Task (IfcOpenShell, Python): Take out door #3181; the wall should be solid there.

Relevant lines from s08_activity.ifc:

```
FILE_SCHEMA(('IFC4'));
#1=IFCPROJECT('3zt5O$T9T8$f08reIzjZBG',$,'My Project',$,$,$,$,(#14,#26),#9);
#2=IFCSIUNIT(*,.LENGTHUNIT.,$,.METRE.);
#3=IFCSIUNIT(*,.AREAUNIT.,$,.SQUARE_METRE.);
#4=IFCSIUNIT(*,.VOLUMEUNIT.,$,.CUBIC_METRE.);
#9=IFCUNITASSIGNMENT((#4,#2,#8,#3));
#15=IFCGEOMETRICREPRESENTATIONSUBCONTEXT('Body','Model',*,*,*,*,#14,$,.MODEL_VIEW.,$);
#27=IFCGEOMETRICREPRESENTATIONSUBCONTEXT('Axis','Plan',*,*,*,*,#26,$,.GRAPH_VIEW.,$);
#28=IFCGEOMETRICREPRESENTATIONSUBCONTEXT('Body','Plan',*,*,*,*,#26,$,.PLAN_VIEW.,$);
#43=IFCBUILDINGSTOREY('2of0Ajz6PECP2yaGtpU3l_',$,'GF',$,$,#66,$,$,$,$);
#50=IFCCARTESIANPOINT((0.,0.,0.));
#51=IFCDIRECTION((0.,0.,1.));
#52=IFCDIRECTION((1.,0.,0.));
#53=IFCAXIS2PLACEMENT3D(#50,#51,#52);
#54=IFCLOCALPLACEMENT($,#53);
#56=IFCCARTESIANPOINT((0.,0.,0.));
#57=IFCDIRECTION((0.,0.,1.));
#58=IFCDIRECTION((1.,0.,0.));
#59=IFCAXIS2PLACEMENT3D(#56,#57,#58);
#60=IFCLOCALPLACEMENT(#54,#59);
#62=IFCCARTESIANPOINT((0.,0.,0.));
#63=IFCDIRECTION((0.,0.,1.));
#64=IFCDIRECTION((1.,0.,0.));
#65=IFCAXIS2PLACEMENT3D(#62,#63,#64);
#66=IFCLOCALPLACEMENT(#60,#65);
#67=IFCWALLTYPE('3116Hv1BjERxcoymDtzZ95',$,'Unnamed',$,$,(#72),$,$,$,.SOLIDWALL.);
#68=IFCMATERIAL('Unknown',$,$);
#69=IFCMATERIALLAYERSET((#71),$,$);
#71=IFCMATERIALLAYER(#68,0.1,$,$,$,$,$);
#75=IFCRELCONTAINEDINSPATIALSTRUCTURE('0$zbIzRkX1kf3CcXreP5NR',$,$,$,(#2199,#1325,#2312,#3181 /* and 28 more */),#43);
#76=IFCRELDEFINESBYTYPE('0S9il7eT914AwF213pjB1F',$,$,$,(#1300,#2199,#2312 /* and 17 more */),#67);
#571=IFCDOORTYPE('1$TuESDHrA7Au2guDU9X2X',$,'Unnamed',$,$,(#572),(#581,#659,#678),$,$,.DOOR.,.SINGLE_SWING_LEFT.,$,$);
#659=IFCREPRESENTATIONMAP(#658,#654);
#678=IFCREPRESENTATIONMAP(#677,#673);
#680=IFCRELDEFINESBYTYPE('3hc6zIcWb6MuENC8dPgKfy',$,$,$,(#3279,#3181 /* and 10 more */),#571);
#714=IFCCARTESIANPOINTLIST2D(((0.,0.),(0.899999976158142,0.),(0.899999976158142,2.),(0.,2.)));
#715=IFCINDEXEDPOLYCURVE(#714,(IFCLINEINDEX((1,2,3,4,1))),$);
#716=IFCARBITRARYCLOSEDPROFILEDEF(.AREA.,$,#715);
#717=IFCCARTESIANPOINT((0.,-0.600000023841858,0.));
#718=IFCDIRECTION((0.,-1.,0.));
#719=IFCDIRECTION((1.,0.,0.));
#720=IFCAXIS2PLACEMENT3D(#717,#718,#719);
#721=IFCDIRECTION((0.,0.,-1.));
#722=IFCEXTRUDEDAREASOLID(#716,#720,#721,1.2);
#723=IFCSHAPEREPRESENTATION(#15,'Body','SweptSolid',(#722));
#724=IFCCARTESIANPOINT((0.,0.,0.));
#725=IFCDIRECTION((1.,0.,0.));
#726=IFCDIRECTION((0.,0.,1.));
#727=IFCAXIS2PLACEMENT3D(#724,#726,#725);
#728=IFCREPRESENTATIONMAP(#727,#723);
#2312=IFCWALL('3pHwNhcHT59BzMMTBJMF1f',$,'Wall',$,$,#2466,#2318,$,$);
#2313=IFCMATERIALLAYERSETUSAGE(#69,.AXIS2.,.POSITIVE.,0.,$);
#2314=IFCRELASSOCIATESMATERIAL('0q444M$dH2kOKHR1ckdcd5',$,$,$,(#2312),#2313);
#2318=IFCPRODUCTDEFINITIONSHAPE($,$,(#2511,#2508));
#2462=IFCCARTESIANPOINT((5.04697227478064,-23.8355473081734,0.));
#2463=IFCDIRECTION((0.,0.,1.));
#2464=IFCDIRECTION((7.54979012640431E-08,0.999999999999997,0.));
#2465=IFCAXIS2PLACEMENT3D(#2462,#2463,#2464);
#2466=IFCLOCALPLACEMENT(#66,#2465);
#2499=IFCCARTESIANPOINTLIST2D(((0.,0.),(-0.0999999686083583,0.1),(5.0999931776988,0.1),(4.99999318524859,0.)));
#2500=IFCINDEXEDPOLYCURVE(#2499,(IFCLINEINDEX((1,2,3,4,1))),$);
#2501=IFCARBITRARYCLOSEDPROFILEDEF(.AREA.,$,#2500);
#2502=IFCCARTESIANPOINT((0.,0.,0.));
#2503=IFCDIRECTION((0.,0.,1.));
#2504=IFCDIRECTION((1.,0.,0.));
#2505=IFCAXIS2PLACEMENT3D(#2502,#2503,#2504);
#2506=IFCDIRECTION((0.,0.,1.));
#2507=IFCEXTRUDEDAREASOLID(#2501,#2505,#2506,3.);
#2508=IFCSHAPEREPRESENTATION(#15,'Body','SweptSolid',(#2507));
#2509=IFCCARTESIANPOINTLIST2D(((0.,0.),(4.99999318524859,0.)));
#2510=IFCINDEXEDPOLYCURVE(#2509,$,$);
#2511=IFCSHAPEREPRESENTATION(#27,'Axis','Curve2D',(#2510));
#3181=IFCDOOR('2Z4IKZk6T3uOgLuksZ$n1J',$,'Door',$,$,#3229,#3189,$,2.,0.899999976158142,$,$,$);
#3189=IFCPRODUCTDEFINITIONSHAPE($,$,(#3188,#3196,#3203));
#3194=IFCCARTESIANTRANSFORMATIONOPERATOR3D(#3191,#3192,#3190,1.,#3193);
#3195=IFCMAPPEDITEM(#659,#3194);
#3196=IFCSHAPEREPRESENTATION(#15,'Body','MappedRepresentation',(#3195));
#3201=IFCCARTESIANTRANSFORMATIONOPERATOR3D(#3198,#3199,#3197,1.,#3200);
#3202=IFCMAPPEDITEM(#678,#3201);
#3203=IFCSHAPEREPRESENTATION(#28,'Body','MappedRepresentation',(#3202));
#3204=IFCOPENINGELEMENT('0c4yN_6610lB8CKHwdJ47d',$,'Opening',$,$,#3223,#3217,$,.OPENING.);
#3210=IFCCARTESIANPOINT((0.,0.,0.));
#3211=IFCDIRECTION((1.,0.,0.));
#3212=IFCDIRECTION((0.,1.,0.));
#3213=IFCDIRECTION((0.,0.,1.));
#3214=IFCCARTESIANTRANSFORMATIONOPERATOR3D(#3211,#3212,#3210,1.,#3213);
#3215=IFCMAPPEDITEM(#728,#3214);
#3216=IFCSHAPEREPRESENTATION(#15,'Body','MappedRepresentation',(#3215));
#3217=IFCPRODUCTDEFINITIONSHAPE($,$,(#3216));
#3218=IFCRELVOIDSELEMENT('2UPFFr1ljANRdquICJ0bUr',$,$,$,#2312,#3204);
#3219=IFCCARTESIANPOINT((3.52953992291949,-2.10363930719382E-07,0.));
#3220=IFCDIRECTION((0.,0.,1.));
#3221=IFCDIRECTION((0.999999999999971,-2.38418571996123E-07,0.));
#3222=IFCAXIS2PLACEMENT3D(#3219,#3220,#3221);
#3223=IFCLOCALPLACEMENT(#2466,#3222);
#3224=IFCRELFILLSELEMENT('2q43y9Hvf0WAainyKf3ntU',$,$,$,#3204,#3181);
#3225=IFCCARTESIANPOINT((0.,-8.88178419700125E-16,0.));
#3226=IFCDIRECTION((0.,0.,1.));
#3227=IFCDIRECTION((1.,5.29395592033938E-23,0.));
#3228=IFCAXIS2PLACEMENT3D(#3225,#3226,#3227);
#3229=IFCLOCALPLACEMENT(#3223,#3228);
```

```python
import ifcopenshell
import ifcopenshell.api.feature
import ifcopenshell.api.root
import ifcopenshell.geom
import ifcopenshell.util.shape

model = ifcopenshell.open("s08_activity.ifc")
settings = ifcopenshell.geom.settings()


def volume(element):
    """Net volume in cubic metres, openings subtracted."""
    shape = ifcopenshell.geom.create_shape(settings, element)
    return ifcopenshell.util.shape.get_volume(shape.geometry)


door = model.by_guid("2Z4IKZk6T3uOgLuksZ$n1J")
opening = door.FillsVoids[0].RelatingOpeningElement
wall = opening.VoidsElements[0].RelatingBuildingElement
before = volume(wall)

ifcopenshell.api.root.remove_product(model, product=door)
ifcopenshell.api.feature.remove_feature(model, feature=opening)

after = volume(wall)

print(f"wall volume {before:.3f} -> {after:.3f} m3")

model.write("s08_activity_rev.ifc")
```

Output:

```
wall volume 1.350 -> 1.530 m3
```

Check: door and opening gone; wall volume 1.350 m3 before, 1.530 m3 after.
